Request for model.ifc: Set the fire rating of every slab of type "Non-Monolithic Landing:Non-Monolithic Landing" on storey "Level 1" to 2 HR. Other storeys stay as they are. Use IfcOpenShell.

First a look at what the model holds.

```python
import ifcopenshell
import ifcopenshell.util.element

model = ifcopenshell.open("model.ifc")
print(model.schema)
storey = next(s for s in model.by_type("IfcBuildingStorey") if s.Name == "Level 1")
slabs = [e for e in ifcopenshell.util.element.get_decomposition(storey) if e.is_a("IfcSlab")]
seen = {}
for e in slabs:
    element_type = ifcopenshell.util.element.get_type(e)
    key = (element_type.Name if element_type != e and element_type else None, ifcopenshell.util.element.get_pset(e, "Pset_SlabCommon", "FireRating"))
    seen[key] = seen.get(key, 0) + 1
for (name, value), count in sorted(seen.items(), key=str):
    print(count, "x", name, "|", value)
```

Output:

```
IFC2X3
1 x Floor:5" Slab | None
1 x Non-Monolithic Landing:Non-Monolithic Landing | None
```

```python
import ifcopenshell
import ifcopenshell.api.pset
import ifcopenshell.util.element

model = ifcopenshell.open("model.ifc")

storey = next(s for s in model.by_type("IfcBuildingStorey") if s.Name == "Level 1")
slabs = [e for e in ifcopenshell.util.element.get_decomposition(storey) if e.is_a("IfcSlab")]

count = 0
for e in slabs:
    element_type = ifcopenshell.util.element.get_type(e)
    if element_type in (None, e) or element_type.Name != "Non-Monolithic Landing:Non-Monolithic Landing":
        continue
    # add_pset returns the element's existing set when there is one.
    pset = ifcopenshell.api.pset.add_pset(model, product=e, name="Pset_SlabCommon")
    ifcopenshell.api.pset.edit_pset(model, pset=pset, properties={"FireRating": "2 HR"})
    count += 1

print(count, "slabs updated")

model.write("model_updated.ifc")
```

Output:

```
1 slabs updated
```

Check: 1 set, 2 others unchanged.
